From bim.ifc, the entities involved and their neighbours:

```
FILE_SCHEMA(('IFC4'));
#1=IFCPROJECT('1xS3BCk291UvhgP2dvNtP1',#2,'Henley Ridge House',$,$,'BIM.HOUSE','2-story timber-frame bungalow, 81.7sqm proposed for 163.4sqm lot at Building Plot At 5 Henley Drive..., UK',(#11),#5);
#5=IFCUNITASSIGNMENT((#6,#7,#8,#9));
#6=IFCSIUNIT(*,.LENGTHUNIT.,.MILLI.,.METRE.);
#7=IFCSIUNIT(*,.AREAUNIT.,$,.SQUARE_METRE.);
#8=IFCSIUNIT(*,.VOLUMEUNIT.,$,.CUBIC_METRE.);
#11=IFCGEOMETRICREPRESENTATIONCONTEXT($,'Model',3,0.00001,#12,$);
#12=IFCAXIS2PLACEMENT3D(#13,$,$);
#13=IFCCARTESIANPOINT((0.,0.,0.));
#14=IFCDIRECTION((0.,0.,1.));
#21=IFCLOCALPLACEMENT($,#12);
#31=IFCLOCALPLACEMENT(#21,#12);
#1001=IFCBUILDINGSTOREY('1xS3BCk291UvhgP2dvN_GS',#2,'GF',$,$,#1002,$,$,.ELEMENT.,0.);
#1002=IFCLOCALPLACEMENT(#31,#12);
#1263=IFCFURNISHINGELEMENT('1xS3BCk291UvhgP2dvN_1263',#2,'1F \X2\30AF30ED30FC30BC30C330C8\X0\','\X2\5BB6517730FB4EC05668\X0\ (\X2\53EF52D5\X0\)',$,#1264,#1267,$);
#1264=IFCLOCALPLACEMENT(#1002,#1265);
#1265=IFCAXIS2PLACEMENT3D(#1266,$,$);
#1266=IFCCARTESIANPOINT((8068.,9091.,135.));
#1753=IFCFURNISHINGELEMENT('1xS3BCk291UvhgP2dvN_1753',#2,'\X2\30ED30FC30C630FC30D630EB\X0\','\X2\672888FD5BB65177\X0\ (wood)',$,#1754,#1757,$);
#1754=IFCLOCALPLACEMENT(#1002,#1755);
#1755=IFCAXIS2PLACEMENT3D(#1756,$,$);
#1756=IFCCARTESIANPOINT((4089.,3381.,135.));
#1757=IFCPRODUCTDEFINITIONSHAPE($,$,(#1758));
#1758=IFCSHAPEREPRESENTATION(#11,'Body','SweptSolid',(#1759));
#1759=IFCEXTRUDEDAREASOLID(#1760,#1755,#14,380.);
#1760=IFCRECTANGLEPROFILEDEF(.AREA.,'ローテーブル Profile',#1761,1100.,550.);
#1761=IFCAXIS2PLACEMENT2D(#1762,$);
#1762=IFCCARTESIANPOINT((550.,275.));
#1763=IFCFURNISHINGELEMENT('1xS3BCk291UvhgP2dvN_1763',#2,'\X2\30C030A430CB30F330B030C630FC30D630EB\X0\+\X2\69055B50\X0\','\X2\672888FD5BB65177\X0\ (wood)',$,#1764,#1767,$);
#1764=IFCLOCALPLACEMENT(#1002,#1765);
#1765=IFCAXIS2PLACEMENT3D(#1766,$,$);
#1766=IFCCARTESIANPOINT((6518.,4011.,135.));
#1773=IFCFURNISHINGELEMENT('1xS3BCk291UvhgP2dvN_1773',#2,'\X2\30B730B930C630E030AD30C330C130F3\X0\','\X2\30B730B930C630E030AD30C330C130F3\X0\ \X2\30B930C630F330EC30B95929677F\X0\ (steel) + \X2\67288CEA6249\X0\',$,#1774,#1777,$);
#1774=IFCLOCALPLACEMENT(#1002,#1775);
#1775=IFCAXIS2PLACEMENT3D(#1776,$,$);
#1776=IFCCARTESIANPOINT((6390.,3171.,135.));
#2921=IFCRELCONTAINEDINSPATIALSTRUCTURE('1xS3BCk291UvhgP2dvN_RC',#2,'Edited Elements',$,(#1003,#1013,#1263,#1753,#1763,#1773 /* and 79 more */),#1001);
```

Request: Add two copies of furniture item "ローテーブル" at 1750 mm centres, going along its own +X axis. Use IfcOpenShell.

```python
import ifcopenshell
import ifcopenshell.api.geometry
import ifcopenshell.api.root
import ifcopenshell.util.element
import ifcopenshell.util.placement
import ifcopenshell.util.unit

model = ifcopenshell.open("bim.ifc")
unit_scale = ifcopenshell.util.unit.calculate_unit_scale(model)


def reuse_history(source, copy):
    """copy_class also copies each property set's owner history, people and application; keep the originals."""
    for rel in copy.IsDefinedBy:
        if rel.is_a("IfcRelDefinesByProperties") and (history := rel.RelatingPropertyDefinition.OwnerHistory):
            rel.RelatingPropertyDefinition.OwnerHistory = source.OwnerHistory
            ifcopenshell.util.element.remove_deep2(model, history)


source = model.by_guid("1xS3BCk291UvhgP2dvN_1753")
base = ifcopenshell.util.placement.get_local_placement(source.ObjectPlacement)
step = base[:3, 0] * 1.75 / unit_scale

for i in range(1, 3):
    copy = ifcopenshell.api.root.copy_class(model, product=source)
    copy.Representation = ifcopenshell.util.element.copy_deep(
        model, source.Representation, exclude=["IfcGeometricRepresentationContext", "IfcRepresentationMap"]
    )
    reuse_history(source, copy)
    matrix = base.copy()
    matrix[:3, 3] += i * step
    print("added at", matrix[:3, 3].round(3) + 0.0)
    ifcopenshell.api.geometry.edit_object_placement(model, product=copy, matrix=matrix, is_si=False)

model.write("bim_v2.ifc")
```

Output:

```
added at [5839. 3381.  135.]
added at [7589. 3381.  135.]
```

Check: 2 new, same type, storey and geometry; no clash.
